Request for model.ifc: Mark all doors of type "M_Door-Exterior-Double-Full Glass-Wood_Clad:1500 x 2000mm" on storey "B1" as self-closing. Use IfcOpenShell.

First a look at what the model holds.

```python
import ifcopenshell
import ifcopenshell.util.element

model = ifcopenshell.open("model.ifc")
print(model.schema)
storey = next(s for s in model.by_type("IfcBuildingStorey") if s.Name == "B1")
doors = [e for e in ifcopenshell.util.element.get_decomposition(storey) if e.is_a("IfcDoor")]
seen = {}
for e in doors:
    element_type = ifcopenshell.util.element.get_type(e)
    key = (element_type.Name if element_type != e and element_type else None, ifcopenshell.util.element.get_pset(e, "Pset_DoorCommon", "SelfClosing"))
    seen[key] = seen.get(key, 0) + 1
for (name, value), count in sorted(seen.items(), key=str):
    print(count, "x", name, "|", value)
```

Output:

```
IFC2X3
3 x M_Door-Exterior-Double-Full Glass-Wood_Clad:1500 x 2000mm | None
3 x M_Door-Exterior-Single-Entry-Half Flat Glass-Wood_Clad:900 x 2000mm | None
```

```python
import ifcopenshell
import ifcopenshell.api.pset
import ifcopenshell.util.element

model = ifcopenshell.open("model.ifc")

storey = next(s for s in model.by_type("IfcBuildingStorey") if s.Name == "B1")
doors = [e for e in ifcopenshell.util.element.get_decomposition(storey) if e.is_a("IfcDoor")]

count = 0
for e in doors:
    element_type = ifcopenshell.util.element.get_type(e)
    if element_type in (None, e) or element_type.Name != "M_Door-Exterior-Double-Full Glass-Wood_Clad:1500 x 2000mm":
        continue
    # add_pset returns the element's existing set when there is one.
    pset = ifcopenshell.api.pset.add_pset(model, product=e, name="Pset_DoorCommon")
    ifcopenshell.api.pset.edit_pset(model, pset=pset, properties={"SelfClosing": True})
    count += 1

print(count, "doors updated")

model.write("model_v2.ifc")
```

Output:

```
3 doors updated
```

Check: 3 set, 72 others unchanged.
